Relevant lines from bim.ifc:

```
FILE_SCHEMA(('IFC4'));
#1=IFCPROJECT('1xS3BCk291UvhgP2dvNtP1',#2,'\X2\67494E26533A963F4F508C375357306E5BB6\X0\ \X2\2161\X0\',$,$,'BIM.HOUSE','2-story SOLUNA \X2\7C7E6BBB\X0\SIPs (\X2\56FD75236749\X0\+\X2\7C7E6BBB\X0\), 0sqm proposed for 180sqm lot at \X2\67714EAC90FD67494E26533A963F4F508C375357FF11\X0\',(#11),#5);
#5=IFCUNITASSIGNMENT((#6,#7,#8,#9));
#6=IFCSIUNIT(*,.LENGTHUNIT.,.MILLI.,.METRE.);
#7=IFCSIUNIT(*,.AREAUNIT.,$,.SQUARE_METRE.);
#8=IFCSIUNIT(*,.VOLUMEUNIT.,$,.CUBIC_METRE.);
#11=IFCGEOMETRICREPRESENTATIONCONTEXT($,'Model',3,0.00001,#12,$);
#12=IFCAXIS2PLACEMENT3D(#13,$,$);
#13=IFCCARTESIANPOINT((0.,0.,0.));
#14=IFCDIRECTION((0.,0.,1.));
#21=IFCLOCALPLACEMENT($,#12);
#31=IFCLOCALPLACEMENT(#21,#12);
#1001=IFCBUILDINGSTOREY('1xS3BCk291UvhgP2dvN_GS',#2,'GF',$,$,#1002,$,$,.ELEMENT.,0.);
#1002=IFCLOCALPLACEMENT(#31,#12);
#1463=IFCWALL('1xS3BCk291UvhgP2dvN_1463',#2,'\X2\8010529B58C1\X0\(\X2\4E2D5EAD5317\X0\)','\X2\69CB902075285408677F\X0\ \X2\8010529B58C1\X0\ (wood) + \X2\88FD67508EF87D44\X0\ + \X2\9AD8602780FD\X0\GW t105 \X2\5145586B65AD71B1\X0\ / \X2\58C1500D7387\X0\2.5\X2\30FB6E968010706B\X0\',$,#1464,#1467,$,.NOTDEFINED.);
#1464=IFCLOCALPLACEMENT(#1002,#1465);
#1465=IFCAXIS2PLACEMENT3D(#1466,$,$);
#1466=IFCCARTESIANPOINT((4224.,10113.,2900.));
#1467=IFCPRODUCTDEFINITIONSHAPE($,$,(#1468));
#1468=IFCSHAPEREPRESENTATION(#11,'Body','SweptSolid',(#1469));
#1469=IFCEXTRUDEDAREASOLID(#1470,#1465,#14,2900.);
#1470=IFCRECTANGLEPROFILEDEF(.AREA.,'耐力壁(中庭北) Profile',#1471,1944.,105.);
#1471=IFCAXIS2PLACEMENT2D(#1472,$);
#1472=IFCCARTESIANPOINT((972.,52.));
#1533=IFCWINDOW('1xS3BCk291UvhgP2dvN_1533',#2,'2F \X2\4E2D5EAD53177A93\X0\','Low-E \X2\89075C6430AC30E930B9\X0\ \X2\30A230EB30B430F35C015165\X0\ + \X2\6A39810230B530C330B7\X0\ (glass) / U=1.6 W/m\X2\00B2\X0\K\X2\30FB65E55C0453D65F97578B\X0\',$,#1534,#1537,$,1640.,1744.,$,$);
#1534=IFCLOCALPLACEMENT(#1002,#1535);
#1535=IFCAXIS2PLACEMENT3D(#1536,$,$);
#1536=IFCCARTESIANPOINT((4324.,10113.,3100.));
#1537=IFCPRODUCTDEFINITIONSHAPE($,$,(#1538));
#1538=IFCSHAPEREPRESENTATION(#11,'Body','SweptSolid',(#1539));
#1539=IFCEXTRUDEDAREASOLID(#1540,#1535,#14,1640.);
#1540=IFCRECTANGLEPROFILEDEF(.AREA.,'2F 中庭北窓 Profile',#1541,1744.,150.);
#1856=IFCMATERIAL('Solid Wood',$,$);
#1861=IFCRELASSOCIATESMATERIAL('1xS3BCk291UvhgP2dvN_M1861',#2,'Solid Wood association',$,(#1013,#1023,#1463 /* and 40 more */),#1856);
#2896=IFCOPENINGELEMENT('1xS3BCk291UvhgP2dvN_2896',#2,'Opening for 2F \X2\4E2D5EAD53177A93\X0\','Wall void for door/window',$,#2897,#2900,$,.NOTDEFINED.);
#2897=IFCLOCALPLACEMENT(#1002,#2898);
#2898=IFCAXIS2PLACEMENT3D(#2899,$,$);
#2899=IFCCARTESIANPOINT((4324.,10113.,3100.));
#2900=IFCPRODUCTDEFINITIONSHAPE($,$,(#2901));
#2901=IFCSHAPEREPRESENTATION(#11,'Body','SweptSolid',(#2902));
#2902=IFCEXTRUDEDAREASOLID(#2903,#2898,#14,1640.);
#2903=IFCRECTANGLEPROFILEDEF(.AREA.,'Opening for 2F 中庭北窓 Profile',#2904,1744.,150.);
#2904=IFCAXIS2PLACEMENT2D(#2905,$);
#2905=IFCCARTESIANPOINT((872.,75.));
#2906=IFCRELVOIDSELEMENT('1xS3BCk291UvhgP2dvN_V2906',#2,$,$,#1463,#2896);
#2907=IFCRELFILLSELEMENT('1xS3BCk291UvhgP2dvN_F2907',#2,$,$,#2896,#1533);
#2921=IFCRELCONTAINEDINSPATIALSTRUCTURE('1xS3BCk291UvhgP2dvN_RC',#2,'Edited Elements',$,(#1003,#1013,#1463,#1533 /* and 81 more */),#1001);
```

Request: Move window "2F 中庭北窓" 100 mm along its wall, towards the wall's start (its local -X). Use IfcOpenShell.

```python
import ifcopenshell
import ifcopenshell.api.geometry
import ifcopenshell.util.placement

model = ifcopenshell.open("bim.ifc")

window = model.by_guid("1xS3BCk291UvhgP2dvN_1533")
opening = window.FillsVoids[0].RelatingOpeningElement
wall = opening.VoidsElements[0].RelatingBuildingElement

wall_matrix = ifcopenshell.util.placement.get_local_placement(wall.ObjectPlacement)
shift = wall_matrix[:3, 0] * -100.0
before = ifcopenshell.util.placement.get_local_placement(window.ObjectPlacement)[:3, 3].copy()

# The window is not placed relative to its opening, so move both.
for product in (opening, window):
    matrix = ifcopenshell.util.placement.get_local_placement(product.ObjectPlacement)
    matrix[:3, 3] += shift
    ifcopenshell.api.geometry.edit_object_placement(model, product=product, matrix=matrix, is_si=False)

after = ifcopenshell.util.placement.get_local_placement(window.ObjectPlacement)[:3, 3]
print("window moved by", (after - before).round(3) + 0.0)

model.write("bim_updated.ifc")
```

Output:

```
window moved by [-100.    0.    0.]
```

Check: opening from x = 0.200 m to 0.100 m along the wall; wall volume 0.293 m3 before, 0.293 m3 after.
